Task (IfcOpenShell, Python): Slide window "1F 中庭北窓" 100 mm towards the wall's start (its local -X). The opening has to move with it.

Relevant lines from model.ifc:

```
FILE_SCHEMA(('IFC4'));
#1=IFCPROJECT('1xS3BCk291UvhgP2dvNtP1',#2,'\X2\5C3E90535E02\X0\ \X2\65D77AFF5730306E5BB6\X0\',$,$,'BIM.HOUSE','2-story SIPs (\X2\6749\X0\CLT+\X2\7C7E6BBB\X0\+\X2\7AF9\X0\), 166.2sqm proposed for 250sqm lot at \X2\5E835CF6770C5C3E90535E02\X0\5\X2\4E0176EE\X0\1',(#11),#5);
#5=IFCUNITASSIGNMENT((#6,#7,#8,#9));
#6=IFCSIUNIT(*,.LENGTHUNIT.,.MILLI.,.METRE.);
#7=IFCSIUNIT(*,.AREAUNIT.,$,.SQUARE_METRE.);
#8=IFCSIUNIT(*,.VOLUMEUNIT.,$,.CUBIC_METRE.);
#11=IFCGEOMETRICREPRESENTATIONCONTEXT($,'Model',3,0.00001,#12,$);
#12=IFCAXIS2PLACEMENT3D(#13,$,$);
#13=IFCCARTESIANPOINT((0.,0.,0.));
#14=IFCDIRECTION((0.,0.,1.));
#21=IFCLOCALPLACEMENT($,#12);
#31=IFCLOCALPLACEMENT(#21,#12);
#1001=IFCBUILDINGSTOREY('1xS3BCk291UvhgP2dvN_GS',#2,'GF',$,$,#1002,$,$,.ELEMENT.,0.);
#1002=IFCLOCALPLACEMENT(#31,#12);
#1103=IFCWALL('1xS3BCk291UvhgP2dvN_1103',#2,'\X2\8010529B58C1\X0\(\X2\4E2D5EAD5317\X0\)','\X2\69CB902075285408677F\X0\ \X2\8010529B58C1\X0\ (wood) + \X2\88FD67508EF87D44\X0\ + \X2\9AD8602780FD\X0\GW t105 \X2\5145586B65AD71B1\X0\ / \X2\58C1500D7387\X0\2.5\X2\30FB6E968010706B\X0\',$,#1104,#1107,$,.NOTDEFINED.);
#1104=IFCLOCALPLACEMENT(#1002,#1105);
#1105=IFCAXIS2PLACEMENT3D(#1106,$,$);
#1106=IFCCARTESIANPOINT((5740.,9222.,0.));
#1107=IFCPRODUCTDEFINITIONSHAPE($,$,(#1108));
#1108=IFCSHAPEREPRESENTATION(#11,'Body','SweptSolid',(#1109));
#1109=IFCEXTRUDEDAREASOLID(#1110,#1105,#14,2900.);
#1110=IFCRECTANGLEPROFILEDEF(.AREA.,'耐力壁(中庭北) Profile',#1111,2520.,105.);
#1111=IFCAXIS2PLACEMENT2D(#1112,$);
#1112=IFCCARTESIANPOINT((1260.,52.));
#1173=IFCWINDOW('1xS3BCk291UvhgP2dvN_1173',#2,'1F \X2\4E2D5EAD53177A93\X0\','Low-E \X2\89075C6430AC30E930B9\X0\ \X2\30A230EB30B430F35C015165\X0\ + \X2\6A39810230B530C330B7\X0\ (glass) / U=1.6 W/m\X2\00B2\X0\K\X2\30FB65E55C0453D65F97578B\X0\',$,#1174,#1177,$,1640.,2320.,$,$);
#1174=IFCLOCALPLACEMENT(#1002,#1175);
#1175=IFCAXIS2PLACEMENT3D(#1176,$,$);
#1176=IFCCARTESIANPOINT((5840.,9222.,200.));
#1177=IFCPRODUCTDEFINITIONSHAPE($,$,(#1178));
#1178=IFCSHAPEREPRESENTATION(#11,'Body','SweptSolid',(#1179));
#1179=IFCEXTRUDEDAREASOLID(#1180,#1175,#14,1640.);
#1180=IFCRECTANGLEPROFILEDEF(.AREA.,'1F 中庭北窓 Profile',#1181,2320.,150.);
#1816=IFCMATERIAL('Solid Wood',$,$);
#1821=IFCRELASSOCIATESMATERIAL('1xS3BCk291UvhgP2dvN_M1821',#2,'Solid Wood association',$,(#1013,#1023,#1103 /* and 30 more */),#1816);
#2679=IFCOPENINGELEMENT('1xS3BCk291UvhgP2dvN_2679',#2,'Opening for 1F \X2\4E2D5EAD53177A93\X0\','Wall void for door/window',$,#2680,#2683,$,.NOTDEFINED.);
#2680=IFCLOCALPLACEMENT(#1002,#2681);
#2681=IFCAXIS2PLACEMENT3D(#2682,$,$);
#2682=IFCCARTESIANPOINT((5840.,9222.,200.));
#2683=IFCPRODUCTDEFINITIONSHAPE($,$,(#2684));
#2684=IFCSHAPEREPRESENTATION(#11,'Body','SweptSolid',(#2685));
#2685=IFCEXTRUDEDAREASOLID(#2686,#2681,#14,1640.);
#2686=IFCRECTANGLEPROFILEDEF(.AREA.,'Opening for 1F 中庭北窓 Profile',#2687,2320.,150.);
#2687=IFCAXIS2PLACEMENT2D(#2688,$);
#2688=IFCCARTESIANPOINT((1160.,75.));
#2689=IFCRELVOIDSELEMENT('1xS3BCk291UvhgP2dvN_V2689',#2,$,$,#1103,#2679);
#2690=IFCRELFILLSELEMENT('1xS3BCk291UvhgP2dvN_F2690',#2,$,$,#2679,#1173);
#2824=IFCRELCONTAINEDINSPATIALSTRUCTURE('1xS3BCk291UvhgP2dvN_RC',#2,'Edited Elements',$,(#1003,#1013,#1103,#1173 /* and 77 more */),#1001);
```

```python
import ifcopenshell
import ifcopenshell.api.geometry
import ifcopenshell.util.placement

model = ifcopenshell.open("model.ifc")

window = model.by_guid("1xS3BCk291UvhgP2dvN_1173")
opening = window.FillsVoids[0].RelatingOpeningElement
wall = opening.VoidsElements[0].RelatingBuildingElement

wall_matrix = ifcopenshell.util.placement.get_local_placement(wall.ObjectPlacement)
shift = wall_matrix[:3, 0] * -100.0
before = ifcopenshell.util.placement.get_local_placement(window.ObjectPlacement)[:3, 3].copy()

# The window is not placed relative to its opening, so move both.
for product in (opening, window):
    matrix = ifcopenshell.util.placement.get_local_placement(product.ObjectPlacement)
    matrix[:3, 3] += shift
    ifcopenshell.api.geometry.edit_object_placement(model, product=product, matrix=matrix, is_si=False)

after = ifcopenshell.util.placement.get_local_placement(window.ObjectPlacement)[:3, 3]
print("window moved by", (after - before).round(3) + 0.0)

model.write("model_rev.ifc")
```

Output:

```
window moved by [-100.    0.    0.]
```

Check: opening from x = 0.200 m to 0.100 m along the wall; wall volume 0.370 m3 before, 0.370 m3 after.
